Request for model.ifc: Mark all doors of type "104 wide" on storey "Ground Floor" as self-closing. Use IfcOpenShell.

First a look at what the model holds.

```python
import ifcopenshell
import ifcopenshell.util.element

model = ifcopenshell.open("model.ifc")
print(model.schema)
storey = next(s for s in model.by_type("IfcBuildingStorey") if s.Name == "Ground Floor")
doors = [e for e in ifcopenshell.util.element.get_decomposition(storey) if e.is_a("IfcDoor")]
seen = {}
for e in doors:
    element_type = ifcopenshell.util.element.get_type(e)
    key = (element_type.Name if element_type != e and element_type else None, ifcopenshell.util.element.get_pset(e, "Pset_DoorCommon", "SelfClosing"))
    seen[key] = seen.get(key, 0) + 1
for (name, value), count in sorted(seen.items(), key=str):
    print(count, "x", name, "|", value)
```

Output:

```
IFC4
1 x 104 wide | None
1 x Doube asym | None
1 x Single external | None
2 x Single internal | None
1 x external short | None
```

```python
import ifcopenshell
import ifcopenshell.api.pset
import ifcopenshell.util.element

model = ifcopenshell.open("model.ifc")

storey = next(s for s in model.by_type("IfcBuildingStorey") if s.Name == "Ground Floor")
doors = [e for e in ifcopenshell.util.element.get_decomposition(storey) if e.is_a("IfcDoor")]

count = 0
for e in doors:
    element_type = ifcopenshell.util.element.get_type(e)
    if element_type in (None, e) or element_type.Name != "104 wide":
        continue
    # add_pset returns the element's existing set when there is one.
    pset = ifcopenshell.api.pset.add_pset(model, product=e, name="Pset_DoorCommon")
    ifcopenshell.api.pset.edit_pset(model, pset=pset, properties={"SelfClosing": True})
    count += 1

print(count, "doors updated")

model.write("model_rev.ifc")
```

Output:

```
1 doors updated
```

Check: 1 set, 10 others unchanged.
